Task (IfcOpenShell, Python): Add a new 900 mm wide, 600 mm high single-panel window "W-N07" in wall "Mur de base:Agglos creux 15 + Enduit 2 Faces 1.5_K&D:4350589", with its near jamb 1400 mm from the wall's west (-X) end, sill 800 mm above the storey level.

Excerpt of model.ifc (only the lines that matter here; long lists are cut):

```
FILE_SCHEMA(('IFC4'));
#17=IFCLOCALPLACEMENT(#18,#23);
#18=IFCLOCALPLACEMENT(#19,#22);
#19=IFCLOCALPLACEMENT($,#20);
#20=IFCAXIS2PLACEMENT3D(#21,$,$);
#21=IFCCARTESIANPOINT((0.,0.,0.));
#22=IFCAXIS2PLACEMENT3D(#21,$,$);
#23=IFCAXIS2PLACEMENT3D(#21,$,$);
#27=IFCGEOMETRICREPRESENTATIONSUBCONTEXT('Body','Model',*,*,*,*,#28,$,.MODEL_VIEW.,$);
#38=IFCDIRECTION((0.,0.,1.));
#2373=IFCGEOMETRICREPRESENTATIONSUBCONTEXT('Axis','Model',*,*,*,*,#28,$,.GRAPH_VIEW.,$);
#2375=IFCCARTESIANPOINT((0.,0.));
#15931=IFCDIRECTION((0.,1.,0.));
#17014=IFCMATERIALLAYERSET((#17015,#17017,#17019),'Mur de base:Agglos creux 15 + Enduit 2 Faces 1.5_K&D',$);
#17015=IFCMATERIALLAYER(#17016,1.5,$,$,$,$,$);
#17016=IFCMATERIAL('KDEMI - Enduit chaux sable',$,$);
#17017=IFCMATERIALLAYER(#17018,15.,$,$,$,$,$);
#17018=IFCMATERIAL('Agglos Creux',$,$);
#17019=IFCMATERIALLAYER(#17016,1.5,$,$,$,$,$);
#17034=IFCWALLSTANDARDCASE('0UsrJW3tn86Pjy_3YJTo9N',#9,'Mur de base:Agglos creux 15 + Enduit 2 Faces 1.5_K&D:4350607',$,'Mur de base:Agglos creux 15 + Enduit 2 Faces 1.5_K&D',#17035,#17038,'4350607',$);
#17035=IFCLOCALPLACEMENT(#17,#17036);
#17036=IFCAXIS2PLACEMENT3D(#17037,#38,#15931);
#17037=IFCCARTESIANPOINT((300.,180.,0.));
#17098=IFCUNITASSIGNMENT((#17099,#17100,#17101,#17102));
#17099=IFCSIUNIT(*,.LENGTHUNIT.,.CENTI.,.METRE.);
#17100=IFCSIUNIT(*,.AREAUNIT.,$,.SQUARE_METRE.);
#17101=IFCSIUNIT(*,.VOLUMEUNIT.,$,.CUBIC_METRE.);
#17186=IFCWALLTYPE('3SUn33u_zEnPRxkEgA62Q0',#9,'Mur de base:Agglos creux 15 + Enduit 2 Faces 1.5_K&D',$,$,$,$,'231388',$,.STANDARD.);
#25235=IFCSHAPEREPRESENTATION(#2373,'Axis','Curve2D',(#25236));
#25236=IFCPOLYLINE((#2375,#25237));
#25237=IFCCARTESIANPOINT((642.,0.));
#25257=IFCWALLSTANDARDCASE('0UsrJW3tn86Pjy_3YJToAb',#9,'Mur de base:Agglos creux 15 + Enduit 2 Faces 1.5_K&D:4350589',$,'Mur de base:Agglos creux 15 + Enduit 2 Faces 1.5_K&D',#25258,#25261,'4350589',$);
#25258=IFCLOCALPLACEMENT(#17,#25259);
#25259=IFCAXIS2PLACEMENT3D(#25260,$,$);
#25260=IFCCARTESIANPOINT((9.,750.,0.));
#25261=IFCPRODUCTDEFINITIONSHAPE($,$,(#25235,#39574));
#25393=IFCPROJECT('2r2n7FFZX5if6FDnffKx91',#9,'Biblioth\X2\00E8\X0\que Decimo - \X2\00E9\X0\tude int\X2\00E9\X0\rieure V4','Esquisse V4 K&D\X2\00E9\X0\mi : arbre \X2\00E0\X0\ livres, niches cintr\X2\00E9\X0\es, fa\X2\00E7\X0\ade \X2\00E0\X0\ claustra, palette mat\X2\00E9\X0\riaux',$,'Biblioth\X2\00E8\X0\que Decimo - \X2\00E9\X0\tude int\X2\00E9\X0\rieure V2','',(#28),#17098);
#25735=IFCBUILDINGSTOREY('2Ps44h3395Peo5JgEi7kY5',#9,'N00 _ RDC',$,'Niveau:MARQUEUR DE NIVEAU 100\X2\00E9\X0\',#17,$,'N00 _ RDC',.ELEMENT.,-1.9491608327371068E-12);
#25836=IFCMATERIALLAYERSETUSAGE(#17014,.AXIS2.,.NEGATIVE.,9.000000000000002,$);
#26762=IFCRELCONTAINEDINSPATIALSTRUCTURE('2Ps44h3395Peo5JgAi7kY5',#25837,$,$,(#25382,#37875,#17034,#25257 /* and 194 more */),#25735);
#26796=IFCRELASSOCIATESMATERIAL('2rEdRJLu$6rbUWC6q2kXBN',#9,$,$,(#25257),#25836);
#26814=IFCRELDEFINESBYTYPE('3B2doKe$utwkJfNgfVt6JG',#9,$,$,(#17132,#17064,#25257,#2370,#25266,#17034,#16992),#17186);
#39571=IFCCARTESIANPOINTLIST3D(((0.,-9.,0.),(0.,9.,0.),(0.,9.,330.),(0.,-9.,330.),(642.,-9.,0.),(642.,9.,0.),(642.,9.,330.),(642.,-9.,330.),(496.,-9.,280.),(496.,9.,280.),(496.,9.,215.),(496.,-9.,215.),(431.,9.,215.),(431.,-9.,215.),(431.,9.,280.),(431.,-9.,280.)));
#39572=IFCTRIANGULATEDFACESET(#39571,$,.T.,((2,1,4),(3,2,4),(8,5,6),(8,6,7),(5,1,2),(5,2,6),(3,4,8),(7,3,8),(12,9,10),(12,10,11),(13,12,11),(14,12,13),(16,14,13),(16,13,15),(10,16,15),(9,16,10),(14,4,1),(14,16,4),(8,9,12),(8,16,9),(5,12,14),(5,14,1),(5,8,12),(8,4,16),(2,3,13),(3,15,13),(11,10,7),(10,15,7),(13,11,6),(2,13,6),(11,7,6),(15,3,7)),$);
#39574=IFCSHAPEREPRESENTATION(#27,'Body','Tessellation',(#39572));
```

```python
import numpy as np
import ifcopenshell
import ifcopenshell.api.feature
import ifcopenshell.api.geometry
import ifcopenshell.api.root
import ifcopenshell.api.spatial
import ifcopenshell.geom
import ifcopenshell.util.element
import ifcopenshell.util.placement
import ifcopenshell.util.representation
import ifcopenshell.util.shape
import ifcopenshell.util.unit

model = ifcopenshell.open("model.ifc")
unit_scale = ifcopenshell.util.unit.calculate_unit_scale(model)
settings = ifcopenshell.geom.settings()


def volume(element):
    """Net volume in cubic metres, openings subtracted."""
    shape = ifcopenshell.geom.create_shape(settings, element)
    return ifcopenshell.util.shape.get_volume(shape.geometry)


wall = model.by_id(25257)
storey = ifcopenshell.util.element.get_container(wall, ifc_class="IfcBuildingStorey")
context = ifcopenshell.util.representation.get_context(model, "Model", "Body", "MODEL_VIEW")
before = volume(wall)

width, height, from_end, sill = 0.9, 0.6, 1.4, 0.8  # metres

# The wall runs along its own X axis, and the end named is its -X end.
wall_shape = ifcopenshell.geom.create_shape(settings, wall)
x, y, z = ifcopenshell.util.shape.get_vertices(wall_shape.geometry).T
start = x.min() + from_end
face, thickness = float(y.min()), float(y.max() - y.min())
wall_matrix = ifcopenshell.util.placement.get_local_placement(wall.ObjectPlacement)
level = ifcopenshell.util.placement.get_local_placement(storey.ObjectPlacement)[2, 3]


def in_wall(x, y):
    """Placement at x, y metres in the wall's axes, at sill height."""
    matrix = wall_matrix.copy()
    matrix[:, 3] = wall_matrix @ np.array([x / unit_scale, y / unit_scale, 0.0, 1.0])
    matrix[2, 3] = level + sill / unit_scale
    return matrix


# Opening: a box that overshoots both wall faces by 50 mm.
opening = ifcopenshell.api.root.create_entity(model, ifc_class="IfcOpeningElement", predefined_type="OPENING")
box = ifcopenshell.api.geometry.add_wall_representation(
    model, context=context, length=width, height=height, thickness=thickness + 0.1
)
ifcopenshell.api.geometry.assign_representation(model, product=opening, representation=box)
ifcopenshell.api.geometry.edit_object_placement(model, product=opening, matrix=in_wall(start, face - 0.05), is_si=False)
ifcopenshell.api.feature.add_feature(model, feature=opening, element=wall)

window = ifcopenshell.api.root.create_entity(model, ifc_class="IfcWindow", name="W-N07", predefined_type="WINDOW")
window.OverallWidth, window.OverallHeight = width / unit_scale, height / unit_scale
window.PartitioningType = "SINGLE_PANEL"
body = ifcopenshell.api.geometry.add_window_representation(
    model,
    context=context,
    overall_width=window.OverallWidth,
    overall_height=window.OverallHeight,
    partition_type="SINGLE_PANEL",
)
ifcopenshell.api.geometry.assign_representation(model, product=window, representation=body)
ifcopenshell.api.spatial.assign_container(model, products=[window], relating_structure=storey)
ifcopenshell.api.feature.add_filling(model, opening=opening, element=window)

# Centre the window in the wall's thickness.
ifcopenshell.api.geometry.edit_object_placement(model, product=window, matrix=in_wall(start, face), is_si=False)
window_shape = ifcopenshell.geom.create_shape(settings, window)
depth = ifcopenshell.util.shape.get_vertices(window_shape.geometry)[:, 1]
offset = face + thickness / 2 - (depth.min() + depth.max()) / 2
ifcopenshell.api.geometry.edit_object_placement(model, product=window, matrix=in_wall(start, offset), is_si=False)

after = volume(wall)

print(f"wall volume {before:.3f} -> {after:.3f} m3")

model.write("model_rev.ifc")
```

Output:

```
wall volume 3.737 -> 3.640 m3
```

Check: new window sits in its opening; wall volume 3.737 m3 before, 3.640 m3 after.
